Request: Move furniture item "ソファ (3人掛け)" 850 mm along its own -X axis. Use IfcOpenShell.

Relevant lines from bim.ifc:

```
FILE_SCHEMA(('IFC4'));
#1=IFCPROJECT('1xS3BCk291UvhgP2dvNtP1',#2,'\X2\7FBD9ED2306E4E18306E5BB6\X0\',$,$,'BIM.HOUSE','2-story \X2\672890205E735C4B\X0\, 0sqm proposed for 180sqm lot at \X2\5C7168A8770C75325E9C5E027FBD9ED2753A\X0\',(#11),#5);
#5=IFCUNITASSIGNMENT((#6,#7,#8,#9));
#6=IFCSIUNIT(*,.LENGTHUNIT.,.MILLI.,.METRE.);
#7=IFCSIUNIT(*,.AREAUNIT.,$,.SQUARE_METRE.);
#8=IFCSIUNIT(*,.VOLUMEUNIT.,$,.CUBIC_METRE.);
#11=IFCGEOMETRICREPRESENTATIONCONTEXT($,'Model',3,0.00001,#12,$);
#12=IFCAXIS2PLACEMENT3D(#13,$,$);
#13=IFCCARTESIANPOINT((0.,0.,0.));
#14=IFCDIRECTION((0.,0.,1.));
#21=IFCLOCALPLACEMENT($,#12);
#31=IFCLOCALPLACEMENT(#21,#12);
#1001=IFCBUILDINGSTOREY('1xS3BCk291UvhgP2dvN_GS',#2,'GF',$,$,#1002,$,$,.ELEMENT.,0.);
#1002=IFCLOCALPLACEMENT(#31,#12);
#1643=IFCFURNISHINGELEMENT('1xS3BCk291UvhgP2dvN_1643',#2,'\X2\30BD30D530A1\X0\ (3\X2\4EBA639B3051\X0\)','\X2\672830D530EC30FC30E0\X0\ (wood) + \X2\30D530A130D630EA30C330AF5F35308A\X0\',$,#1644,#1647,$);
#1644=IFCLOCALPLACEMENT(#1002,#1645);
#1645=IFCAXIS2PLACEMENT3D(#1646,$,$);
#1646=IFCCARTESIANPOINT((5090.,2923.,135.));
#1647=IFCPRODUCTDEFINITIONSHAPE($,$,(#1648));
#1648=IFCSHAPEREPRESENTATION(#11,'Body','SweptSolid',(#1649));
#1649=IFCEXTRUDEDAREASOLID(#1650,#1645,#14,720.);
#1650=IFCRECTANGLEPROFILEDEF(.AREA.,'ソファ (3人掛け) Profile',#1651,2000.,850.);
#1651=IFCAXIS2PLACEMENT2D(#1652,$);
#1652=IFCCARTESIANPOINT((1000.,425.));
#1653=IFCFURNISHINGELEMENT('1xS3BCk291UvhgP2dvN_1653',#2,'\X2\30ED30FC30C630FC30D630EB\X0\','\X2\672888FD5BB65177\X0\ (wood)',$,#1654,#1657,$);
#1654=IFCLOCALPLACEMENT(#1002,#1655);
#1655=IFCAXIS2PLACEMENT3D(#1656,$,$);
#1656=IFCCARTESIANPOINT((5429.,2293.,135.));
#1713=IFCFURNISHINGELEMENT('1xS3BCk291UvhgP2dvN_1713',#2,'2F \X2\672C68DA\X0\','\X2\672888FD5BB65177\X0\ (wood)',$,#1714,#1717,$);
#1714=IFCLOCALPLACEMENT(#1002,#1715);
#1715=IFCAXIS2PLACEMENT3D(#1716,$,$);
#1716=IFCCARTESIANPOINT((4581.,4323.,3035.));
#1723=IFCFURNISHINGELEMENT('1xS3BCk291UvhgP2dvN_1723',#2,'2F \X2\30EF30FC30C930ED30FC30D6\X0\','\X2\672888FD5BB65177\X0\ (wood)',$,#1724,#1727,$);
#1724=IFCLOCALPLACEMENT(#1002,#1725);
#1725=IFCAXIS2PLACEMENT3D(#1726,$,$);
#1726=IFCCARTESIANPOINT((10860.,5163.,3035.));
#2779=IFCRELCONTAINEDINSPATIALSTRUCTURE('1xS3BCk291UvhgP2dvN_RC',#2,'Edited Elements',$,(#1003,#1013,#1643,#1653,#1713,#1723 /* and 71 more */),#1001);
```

```python
import ifcopenshell
import ifcopenshell.api.geometry
import ifcopenshell.util.placement
import ifcopenshell.util.unit

model = ifcopenshell.open("bim.ifc")
unit_scale = ifcopenshell.util.unit.calculate_unit_scale(model)

item = model.by_guid("1xS3BCk291UvhgP2dvN_1643")
matrix = ifcopenshell.util.placement.get_local_placement(item.ObjectPlacement)
matrix[:3, 3] -= matrix[:3, 0] * 0.85 / unit_scale
ifcopenshell.api.geometry.edit_object_placement(model, product=item, matrix=matrix, is_si=False)

print(ifcopenshell.util.placement.get_local_placement(item.ObjectPlacement).round(3) + 0.0)

model.write("bim_v2.ifc")
```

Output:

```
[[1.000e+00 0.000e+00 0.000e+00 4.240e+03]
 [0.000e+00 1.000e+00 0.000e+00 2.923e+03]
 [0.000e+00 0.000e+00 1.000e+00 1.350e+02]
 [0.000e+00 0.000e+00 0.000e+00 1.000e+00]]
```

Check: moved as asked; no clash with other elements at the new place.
